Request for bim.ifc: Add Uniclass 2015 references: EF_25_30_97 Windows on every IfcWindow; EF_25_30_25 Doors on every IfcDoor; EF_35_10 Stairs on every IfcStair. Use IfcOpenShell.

First a look at what the model holds.

```python
import ifcopenshell

model = ifcopenshell.open("bim.ifc")
print(model.schema)
print("classifications:", [c.Name for c in model.by_type("IfcClassification")])
for ifc_class in ("IfcDoor", "IfcRoof", "IfcStair", "IfcWall", "IfcWindow"):
    print(ifc_class, len(model.by_type(ifc_class)))
```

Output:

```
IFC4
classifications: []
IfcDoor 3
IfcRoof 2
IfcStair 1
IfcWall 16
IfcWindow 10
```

```python
import ifcopenshell
import ifcopenshell.api.classification

model = ifcopenshell.open("bim.ifc")

system = ifcopenshell.api.classification.add_classification(model, classification="Uniclass 2015")

codes = {
    "IfcWindow": ("EF_25_30_97", "Windows"),
    "IfcDoor": ("EF_25_30_25", "Doors"),
    "IfcStair": ("EF_35_10", "Stairs"),
}
for ifc_class, (code, name) in codes.items():
    products = model.by_type(ifc_class)
    ifcopenshell.api.classification.add_reference(
        model, products=products, classification=system, identification=code, name=name
    )
    print(code, len(products))

model.write("bim-out.ifc")
```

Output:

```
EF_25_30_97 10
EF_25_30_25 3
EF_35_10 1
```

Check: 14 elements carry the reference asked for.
